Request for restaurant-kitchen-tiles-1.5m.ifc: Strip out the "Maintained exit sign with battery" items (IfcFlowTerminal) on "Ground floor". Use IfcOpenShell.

First a look at what the model holds.

```python
import ifcopenshell
import ifcopenshell.util.element

model = ifcopenshell.open("restaurant-kitchen-tiles-1.5m.ifc")
print(model.schema)
storey = next(s for s in model.by_type("IfcBuildingStorey") if s.Name == "Ground floor")
terminals = [e for e in ifcopenshell.util.element.get_decomposition(storey) if e.is_a("IfcFlowTerminal")]
seen = {}
for e in terminals:
    element_type = ifcopenshell.util.element.get_type(e)
    name = element_type.Name if element_type not in (None, e) else None
    seen[name] = seen.get(name, 0) + 1
for name, count in sorted(seen.items(), key=str):
    print(count, "x", name)
```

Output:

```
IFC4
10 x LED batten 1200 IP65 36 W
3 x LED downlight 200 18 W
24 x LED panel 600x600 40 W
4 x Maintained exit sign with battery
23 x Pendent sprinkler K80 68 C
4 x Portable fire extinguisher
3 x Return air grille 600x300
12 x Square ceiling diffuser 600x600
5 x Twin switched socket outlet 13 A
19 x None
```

```python
import ifcopenshell
import ifcopenshell.api.root
import ifcopenshell.util.element

model = ifcopenshell.open("restaurant-kitchen-tiles-1.5m.ifc")

storey = next(s for s in model.by_type("IfcBuildingStorey") if s.Name == "Ground floor")
terminals = [e for e in ifcopenshell.util.element.get_decomposition(storey) if e.is_a("IfcFlowTerminal")]
targets = [e for e in terminals if (t := ifcopenshell.util.element.get_type(e)) not in (None, e) and t.Name == "Maintained exit sign with battery"]

for e in targets:
    ifcopenshell.api.root.remove_product(model, product=e)
print(len(targets), "removed")

model.write("restaurant-kitchen-tiles-1.5m-out.ifc")
```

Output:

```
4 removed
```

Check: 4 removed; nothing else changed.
